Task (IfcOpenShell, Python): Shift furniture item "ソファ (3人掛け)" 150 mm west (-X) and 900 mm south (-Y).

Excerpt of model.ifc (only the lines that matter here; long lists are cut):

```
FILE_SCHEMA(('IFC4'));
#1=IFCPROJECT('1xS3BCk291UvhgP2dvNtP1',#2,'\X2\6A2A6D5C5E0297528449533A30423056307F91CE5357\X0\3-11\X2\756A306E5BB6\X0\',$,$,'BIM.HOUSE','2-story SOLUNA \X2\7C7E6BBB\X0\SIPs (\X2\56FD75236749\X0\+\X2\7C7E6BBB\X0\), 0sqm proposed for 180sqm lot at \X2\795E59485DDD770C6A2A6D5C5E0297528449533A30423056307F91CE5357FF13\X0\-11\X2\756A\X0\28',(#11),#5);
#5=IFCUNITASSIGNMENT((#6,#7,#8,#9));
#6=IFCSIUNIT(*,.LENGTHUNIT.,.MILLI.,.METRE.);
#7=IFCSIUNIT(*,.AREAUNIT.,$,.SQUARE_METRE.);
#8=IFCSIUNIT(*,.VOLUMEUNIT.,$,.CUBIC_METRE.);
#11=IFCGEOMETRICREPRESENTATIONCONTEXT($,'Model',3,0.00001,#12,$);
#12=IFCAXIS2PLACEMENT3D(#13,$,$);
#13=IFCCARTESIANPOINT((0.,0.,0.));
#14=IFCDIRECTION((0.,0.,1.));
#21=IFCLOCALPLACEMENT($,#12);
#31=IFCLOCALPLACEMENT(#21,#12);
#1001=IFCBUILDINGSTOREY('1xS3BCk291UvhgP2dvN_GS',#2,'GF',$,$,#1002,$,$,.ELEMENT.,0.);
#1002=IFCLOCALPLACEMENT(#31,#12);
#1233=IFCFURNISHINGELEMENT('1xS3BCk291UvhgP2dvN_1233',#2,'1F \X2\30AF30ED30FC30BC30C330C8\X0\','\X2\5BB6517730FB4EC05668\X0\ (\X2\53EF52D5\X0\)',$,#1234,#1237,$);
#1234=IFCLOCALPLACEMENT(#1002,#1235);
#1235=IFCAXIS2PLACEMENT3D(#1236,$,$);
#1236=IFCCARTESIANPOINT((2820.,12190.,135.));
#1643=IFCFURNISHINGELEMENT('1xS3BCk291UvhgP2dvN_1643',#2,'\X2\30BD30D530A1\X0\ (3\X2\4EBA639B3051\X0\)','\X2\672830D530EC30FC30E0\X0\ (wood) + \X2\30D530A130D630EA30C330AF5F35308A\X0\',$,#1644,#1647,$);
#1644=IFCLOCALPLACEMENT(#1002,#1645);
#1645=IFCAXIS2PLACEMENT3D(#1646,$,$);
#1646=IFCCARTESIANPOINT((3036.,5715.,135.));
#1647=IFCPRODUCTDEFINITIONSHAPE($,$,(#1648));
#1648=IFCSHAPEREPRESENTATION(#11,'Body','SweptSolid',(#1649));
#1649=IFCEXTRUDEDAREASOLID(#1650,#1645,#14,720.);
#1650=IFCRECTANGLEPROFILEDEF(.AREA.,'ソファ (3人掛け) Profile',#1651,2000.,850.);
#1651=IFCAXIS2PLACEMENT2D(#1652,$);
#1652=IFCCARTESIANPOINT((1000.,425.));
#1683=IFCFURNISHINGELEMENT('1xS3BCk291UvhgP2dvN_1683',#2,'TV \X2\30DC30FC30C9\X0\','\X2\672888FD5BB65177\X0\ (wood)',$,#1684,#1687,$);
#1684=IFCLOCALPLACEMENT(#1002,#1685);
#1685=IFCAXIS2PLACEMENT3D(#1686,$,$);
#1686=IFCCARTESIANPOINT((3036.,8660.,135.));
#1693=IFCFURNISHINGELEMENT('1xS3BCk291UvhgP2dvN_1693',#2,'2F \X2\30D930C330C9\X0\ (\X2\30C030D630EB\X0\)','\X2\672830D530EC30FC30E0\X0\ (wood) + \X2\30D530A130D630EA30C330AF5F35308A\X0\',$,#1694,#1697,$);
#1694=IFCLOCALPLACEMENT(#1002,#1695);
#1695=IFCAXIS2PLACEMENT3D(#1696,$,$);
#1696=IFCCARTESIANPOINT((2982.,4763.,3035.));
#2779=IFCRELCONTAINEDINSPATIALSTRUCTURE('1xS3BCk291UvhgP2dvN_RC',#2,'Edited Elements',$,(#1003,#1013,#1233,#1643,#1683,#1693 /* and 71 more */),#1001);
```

```python
import ifcopenshell
import ifcopenshell.api.geometry
import ifcopenshell.util.placement

model = ifcopenshell.open("model.ifc")

item = model.by_guid("1xS3BCk291UvhgP2dvN_1643")
matrix = ifcopenshell.util.placement.get_local_placement(item.ObjectPlacement)
matrix[0, 3] -= 150.0
matrix[1, 3] -= 900.0
ifcopenshell.api.geometry.edit_object_placement(model, product=item, matrix=matrix, is_si=False)

print(ifcopenshell.util.placement.get_local_placement(item.ObjectPlacement).round(3) + 0.0)

model.write("model_rev.ifc")
```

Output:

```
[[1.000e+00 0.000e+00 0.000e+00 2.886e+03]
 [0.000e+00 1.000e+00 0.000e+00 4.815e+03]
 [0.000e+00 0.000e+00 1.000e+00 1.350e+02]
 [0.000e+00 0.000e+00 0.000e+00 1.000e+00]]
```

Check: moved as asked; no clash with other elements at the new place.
